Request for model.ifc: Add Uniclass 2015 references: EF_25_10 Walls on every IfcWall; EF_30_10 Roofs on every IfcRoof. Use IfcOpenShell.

First a look at what the model holds.

```python
import ifcopenshell

model = ifcopenshell.open("model.ifc")
print(model.schema)
print("classifications:", [c.Name for c in model.by_type("IfcClassification")])
for ifc_class in ("IfcDoor", "IfcRoof", "IfcStair", "IfcWall", "IfcWindow"):
    print(ifc_class, len(model.by_type(ifc_class)))
```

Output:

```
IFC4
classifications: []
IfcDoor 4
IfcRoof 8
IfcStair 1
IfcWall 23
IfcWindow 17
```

```python
import ifcopenshell
import ifcopenshell.api.classification

model = ifcopenshell.open("model.ifc")

system = ifcopenshell.api.classification.add_classification(model, classification="Uniclass 2015")

codes = {
    "IfcWall": ("EF_25_10", "Walls"),
    "IfcRoof": ("EF_30_10", "Roofs"),
}
for ifc_class, (code, name) in codes.items():
    products = model.by_type(ifc_class)
    ifcopenshell.api.classification.add_reference(
        model, products=products, classification=system, identification=code, name=name
    )
    print(code, len(products))

model.write("model_edited.ifc")
```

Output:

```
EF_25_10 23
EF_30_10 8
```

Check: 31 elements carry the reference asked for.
